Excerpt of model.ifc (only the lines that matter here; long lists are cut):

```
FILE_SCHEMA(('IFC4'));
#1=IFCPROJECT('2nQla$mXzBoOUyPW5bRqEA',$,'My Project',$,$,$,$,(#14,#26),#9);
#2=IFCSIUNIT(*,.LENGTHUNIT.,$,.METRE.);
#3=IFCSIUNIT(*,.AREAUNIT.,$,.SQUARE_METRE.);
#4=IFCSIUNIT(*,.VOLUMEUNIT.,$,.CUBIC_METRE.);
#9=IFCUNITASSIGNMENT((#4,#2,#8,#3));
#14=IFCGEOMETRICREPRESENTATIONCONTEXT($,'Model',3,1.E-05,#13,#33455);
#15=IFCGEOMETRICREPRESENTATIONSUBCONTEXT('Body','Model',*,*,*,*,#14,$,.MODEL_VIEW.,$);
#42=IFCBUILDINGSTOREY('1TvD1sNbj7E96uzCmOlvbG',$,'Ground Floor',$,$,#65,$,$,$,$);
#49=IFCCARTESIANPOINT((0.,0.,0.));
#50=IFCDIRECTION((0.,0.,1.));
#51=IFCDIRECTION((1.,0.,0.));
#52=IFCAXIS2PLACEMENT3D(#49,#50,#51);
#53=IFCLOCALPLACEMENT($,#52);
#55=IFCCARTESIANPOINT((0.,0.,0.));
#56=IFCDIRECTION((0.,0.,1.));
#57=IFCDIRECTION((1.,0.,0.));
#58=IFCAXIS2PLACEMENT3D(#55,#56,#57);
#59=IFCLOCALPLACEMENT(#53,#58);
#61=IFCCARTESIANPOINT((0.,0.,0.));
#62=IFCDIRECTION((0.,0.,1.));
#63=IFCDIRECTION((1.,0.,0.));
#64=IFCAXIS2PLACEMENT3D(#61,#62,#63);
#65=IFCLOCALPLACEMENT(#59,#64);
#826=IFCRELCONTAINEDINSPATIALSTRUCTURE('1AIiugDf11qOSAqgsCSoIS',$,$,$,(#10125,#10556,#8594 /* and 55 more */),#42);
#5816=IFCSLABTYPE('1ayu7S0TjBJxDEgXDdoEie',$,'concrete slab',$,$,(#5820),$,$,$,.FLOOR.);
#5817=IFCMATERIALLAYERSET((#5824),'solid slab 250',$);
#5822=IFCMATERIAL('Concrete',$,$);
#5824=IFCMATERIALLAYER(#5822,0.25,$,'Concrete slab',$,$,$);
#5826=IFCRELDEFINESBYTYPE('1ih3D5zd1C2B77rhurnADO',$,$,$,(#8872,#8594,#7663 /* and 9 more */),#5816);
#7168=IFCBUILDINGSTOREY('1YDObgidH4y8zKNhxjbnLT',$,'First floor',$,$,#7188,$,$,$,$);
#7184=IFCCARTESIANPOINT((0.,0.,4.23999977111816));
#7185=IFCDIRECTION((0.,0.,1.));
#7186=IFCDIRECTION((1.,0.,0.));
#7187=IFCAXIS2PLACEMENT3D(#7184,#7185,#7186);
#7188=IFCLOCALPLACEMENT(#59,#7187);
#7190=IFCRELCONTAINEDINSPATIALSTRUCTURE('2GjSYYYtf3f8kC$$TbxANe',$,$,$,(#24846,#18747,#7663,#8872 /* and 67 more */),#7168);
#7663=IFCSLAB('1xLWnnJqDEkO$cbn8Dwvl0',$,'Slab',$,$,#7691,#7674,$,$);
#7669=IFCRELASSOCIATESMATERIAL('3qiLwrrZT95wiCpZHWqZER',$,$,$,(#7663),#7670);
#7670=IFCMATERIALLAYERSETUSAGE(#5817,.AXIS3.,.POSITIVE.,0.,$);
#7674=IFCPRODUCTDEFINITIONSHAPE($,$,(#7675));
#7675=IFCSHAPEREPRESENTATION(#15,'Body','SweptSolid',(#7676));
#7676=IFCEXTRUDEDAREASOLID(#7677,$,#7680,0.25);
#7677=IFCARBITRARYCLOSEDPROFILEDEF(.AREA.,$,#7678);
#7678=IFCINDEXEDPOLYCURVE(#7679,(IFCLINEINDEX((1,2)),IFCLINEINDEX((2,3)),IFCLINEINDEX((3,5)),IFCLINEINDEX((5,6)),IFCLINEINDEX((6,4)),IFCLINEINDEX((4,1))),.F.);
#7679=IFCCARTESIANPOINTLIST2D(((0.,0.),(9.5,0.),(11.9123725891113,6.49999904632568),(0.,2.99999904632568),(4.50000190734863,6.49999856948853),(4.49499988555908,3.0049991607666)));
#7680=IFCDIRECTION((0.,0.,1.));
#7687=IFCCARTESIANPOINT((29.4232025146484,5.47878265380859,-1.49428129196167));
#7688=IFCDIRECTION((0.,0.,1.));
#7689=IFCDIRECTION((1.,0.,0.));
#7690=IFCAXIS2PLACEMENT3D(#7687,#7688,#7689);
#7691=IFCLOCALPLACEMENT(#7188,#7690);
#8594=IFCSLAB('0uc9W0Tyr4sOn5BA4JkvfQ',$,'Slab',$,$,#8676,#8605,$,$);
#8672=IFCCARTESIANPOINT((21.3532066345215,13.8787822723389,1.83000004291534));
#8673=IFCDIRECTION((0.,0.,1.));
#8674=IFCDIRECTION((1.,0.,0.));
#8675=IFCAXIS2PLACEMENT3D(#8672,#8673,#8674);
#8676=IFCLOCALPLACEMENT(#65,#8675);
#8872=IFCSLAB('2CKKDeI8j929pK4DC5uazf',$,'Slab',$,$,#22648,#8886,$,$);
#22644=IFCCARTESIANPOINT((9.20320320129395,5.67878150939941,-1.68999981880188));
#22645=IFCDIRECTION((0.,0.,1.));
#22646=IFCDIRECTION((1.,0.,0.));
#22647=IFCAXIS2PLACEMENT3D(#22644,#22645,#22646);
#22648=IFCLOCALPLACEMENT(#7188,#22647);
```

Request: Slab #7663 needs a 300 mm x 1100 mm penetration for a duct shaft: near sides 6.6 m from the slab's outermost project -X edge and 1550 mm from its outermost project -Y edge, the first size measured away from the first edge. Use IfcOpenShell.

```python
import numpy as np
import ifcopenshell
import ifcopenshell.api.feature
import ifcopenshell.api.geometry
import ifcopenshell.api.root
import ifcopenshell.geom
import ifcopenshell.util.placement
import ifcopenshell.util.representation
import ifcopenshell.util.shape
import ifcopenshell.util.unit

model = ifcopenshell.open("model.ifc")
unit_scale = ifcopenshell.util.unit.calculate_unit_scale(model)
settings = ifcopenshell.geom.settings()


def volume(element):
    """Net volume in cubic metres, openings subtracted."""
    shape = ifcopenshell.geom.create_shape(settings, element)
    return ifcopenshell.util.shape.get_volume(shape.geometry)


slab = model.by_guid("1xLWnnJqDEkO$cbn8Dwvl0")
before = volume(slab)

# Extent in the slab's own axes, in metres. The edges named are its -X and -Y sides.
slab_shape = ifcopenshell.geom.create_shape(settings, slab)
vertices = ifcopenshell.util.shape.get_vertices(slab_shape.geometry)
x_min, y_min, bottom = vertices.min(axis=0)
top = vertices[:, 2].max()

opening = ifcopenshell.api.root.create_entity(model, ifc_class="IfcOpeningElement", name="Duct shaft opening", predefined_type="OPENING")
context = ifcopenshell.util.representation.get_context(model, "Model", "Body", "MODEL_VIEW")
width, depth = 0.3, 1.1
outline = [(0.0, 0.0), (width, 0.0), (width, depth), (0.0, depth), (0.0, 0.0)]
# Overshoot both faces by 50 mm so the cut is clean.
shape = ifcopenshell.api.geometry.add_slab_representation(
    model, context=context, depth=top - bottom + 0.1, polyline=outline
)
ifcopenshell.api.geometry.assign_representation(model, product=opening, representation=shape)

matrix = ifcopenshell.util.placement.get_local_placement(slab.ObjectPlacement)
matrix[:, 3] = matrix @ np.append(np.array([x_min + 6.6, y_min + 1.55, bottom - 0.05]) / unit_scale, 1.0)
ifcopenshell.api.geometry.edit_object_placement(model, product=opening, matrix=matrix, is_si=False)
ifcopenshell.api.feature.add_feature(model, feature=opening, element=slab)

after = volume(slab)

print(f"slab volume {before:.3f} -> {after:.3f} m3")

model.write("model_rev.ifc")
```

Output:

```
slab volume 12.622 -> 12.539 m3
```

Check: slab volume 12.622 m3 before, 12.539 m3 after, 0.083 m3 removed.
